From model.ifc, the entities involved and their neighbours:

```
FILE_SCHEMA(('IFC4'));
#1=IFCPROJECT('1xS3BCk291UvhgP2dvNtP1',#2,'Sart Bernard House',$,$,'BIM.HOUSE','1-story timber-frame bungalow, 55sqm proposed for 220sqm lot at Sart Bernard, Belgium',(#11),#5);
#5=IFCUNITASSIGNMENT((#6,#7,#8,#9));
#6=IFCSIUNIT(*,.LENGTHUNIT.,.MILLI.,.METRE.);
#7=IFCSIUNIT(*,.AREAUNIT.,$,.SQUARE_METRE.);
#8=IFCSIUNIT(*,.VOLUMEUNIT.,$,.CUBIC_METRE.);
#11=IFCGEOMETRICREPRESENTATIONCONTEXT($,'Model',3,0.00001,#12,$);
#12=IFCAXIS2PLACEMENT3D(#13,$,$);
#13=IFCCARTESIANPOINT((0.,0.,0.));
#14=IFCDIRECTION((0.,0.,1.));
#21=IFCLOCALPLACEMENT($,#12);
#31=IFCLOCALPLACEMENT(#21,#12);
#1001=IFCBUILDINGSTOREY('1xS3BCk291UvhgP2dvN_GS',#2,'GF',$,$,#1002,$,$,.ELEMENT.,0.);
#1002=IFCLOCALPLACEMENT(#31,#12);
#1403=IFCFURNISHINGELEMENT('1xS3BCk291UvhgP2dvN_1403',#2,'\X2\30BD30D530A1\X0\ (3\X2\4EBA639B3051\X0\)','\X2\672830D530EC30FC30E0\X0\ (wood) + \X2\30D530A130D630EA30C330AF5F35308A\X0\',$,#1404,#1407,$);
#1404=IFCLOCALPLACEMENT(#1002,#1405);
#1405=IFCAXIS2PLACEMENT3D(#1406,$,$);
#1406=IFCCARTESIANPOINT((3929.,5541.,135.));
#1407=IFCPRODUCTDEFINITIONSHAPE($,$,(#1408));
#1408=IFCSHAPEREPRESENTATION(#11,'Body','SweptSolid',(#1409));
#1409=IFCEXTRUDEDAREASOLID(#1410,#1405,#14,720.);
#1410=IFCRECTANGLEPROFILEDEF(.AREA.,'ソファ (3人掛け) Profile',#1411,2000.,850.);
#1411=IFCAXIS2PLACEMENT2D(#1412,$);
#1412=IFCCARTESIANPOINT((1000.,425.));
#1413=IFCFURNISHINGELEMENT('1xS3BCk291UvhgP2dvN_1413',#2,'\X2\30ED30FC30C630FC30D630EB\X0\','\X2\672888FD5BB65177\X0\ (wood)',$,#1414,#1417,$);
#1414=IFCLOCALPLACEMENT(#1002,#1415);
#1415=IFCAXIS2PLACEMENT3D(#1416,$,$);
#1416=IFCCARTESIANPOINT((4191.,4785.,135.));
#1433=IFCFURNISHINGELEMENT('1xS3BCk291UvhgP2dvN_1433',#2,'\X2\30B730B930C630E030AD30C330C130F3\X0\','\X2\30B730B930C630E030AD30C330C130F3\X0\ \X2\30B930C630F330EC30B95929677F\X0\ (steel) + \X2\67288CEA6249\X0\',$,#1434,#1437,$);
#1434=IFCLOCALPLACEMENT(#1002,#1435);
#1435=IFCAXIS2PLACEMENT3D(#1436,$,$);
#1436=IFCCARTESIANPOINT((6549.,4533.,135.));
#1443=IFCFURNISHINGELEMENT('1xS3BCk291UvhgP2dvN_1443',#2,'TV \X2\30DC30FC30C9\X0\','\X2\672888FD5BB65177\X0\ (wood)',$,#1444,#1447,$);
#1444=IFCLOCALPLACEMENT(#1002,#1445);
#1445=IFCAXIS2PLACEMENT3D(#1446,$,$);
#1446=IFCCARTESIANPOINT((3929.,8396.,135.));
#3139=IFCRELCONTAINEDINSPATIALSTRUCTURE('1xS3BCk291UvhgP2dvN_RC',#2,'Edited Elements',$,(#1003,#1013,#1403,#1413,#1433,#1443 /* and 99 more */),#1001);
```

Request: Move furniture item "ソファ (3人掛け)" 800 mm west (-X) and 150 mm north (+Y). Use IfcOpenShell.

```python
import ifcopenshell
import ifcopenshell.api.geometry
import ifcopenshell.util.placement
import ifcopenshell.util.unit

model = ifcopenshell.open("model.ifc")
unit_scale = ifcopenshell.util.unit.calculate_unit_scale(model)

item = model.by_guid("1xS3BCk291UvhgP2dvN_1403")
matrix = ifcopenshell.util.placement.get_local_placement(item.ObjectPlacement)
matrix[0, 3] -= 0.8 / unit_scale
matrix[1, 3] += 0.15 / unit_scale
ifcopenshell.api.geometry.edit_object_placement(model, product=item, matrix=matrix, is_si=False)

print(ifcopenshell.util.placement.get_local_placement(item.ObjectPlacement).round(3) + 0.0)

model.write("model_updated.ifc")
```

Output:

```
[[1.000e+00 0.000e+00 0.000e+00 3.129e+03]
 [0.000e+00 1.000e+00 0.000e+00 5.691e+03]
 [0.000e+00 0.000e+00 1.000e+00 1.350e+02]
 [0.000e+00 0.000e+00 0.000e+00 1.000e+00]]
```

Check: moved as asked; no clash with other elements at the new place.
